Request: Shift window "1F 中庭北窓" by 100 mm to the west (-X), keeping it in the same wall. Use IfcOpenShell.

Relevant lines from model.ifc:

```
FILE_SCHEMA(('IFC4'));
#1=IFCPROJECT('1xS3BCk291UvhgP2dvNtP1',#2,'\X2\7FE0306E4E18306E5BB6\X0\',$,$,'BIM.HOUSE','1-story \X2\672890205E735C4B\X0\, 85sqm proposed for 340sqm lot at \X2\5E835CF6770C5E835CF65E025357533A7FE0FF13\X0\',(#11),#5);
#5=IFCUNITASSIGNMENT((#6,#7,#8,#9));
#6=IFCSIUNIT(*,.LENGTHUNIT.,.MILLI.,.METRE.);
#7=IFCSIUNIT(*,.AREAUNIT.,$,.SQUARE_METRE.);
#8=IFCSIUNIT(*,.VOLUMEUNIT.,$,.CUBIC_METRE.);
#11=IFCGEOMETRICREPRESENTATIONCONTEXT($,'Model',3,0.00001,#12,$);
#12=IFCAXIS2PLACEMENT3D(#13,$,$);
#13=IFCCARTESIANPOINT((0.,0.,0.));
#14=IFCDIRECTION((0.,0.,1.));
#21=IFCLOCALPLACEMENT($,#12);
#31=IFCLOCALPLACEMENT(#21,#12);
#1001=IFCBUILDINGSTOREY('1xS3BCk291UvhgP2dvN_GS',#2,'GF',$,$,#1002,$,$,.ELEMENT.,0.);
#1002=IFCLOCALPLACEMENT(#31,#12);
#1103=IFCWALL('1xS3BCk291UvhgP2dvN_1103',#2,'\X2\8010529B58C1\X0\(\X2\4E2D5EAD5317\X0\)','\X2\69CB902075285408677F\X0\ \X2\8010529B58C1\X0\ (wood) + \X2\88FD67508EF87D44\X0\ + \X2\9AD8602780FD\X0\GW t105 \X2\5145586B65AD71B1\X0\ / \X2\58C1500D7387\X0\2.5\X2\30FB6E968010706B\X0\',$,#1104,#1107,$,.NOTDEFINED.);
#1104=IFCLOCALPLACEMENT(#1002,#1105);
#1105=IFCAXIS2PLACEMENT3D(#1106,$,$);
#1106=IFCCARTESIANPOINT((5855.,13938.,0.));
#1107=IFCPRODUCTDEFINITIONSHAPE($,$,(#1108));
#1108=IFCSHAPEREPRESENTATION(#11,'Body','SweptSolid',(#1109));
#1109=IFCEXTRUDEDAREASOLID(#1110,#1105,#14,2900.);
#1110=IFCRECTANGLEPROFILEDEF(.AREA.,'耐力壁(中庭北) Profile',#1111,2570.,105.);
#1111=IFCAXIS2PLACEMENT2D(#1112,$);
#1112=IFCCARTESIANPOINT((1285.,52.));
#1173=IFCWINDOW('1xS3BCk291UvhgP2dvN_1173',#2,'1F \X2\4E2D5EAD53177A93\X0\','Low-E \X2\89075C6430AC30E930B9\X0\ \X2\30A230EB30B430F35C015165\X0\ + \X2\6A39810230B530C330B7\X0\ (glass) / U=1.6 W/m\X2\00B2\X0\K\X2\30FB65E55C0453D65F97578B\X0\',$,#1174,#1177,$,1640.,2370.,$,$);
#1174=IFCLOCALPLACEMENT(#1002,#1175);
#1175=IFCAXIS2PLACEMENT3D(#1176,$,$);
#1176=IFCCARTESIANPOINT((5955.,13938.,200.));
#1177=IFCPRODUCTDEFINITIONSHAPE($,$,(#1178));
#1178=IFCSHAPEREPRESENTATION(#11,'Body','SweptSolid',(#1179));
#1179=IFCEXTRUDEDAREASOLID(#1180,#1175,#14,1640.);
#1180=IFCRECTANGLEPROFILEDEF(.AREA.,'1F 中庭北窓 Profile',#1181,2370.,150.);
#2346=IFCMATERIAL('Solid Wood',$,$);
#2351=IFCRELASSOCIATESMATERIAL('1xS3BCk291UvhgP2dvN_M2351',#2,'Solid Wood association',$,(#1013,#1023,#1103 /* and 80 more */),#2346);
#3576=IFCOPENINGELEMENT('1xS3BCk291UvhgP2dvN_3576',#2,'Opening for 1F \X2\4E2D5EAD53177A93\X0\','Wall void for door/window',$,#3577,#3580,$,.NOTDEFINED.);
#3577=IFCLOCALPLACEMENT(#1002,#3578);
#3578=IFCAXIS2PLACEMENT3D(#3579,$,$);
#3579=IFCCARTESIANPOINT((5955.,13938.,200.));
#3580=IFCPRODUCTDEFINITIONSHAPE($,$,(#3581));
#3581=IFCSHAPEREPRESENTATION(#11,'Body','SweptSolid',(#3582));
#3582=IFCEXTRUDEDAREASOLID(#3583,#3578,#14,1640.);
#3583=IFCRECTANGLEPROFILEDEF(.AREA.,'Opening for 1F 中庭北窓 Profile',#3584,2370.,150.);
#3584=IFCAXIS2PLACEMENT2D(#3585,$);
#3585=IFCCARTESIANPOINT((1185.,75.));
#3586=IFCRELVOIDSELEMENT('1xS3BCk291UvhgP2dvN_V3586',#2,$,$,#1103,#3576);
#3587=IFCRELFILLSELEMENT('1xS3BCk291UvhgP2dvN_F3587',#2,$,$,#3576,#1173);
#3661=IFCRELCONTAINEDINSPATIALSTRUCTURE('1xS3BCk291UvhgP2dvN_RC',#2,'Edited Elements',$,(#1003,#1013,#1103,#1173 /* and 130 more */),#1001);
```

```python
import ifcopenshell
import ifcopenshell.api.geometry
import ifcopenshell.util.placement

model = ifcopenshell.open("model.ifc")

window = model.by_guid("1xS3BCk291UvhgP2dvN_1173")
opening = window.FillsVoids[0].RelatingOpeningElement
wall = opening.VoidsElements[0].RelatingBuildingElement

wall_matrix = ifcopenshell.util.placement.get_local_placement(wall.ObjectPlacement)
shift = wall_matrix[:3, 0] * -100.0
before = ifcopenshell.util.placement.get_local_placement(window.ObjectPlacement)[:3, 3].copy()

# The window is not placed relative to its opening, so move both.
for product in (opening, window):
    matrix = ifcopenshell.util.placement.get_local_placement(product.ObjectPlacement)
    matrix[:3, 3] += shift
    ifcopenshell.api.geometry.edit_object_placement(model, product=product, matrix=matrix, is_si=False)

after = ifcopenshell.util.placement.get_local_placement(window.ObjectPlacement)[:3, 3]
print("window moved by", (after - before).round(3) + 0.0)

model.write("model_updated.ifc")
```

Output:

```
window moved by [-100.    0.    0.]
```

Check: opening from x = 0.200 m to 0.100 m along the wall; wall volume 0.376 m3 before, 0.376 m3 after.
